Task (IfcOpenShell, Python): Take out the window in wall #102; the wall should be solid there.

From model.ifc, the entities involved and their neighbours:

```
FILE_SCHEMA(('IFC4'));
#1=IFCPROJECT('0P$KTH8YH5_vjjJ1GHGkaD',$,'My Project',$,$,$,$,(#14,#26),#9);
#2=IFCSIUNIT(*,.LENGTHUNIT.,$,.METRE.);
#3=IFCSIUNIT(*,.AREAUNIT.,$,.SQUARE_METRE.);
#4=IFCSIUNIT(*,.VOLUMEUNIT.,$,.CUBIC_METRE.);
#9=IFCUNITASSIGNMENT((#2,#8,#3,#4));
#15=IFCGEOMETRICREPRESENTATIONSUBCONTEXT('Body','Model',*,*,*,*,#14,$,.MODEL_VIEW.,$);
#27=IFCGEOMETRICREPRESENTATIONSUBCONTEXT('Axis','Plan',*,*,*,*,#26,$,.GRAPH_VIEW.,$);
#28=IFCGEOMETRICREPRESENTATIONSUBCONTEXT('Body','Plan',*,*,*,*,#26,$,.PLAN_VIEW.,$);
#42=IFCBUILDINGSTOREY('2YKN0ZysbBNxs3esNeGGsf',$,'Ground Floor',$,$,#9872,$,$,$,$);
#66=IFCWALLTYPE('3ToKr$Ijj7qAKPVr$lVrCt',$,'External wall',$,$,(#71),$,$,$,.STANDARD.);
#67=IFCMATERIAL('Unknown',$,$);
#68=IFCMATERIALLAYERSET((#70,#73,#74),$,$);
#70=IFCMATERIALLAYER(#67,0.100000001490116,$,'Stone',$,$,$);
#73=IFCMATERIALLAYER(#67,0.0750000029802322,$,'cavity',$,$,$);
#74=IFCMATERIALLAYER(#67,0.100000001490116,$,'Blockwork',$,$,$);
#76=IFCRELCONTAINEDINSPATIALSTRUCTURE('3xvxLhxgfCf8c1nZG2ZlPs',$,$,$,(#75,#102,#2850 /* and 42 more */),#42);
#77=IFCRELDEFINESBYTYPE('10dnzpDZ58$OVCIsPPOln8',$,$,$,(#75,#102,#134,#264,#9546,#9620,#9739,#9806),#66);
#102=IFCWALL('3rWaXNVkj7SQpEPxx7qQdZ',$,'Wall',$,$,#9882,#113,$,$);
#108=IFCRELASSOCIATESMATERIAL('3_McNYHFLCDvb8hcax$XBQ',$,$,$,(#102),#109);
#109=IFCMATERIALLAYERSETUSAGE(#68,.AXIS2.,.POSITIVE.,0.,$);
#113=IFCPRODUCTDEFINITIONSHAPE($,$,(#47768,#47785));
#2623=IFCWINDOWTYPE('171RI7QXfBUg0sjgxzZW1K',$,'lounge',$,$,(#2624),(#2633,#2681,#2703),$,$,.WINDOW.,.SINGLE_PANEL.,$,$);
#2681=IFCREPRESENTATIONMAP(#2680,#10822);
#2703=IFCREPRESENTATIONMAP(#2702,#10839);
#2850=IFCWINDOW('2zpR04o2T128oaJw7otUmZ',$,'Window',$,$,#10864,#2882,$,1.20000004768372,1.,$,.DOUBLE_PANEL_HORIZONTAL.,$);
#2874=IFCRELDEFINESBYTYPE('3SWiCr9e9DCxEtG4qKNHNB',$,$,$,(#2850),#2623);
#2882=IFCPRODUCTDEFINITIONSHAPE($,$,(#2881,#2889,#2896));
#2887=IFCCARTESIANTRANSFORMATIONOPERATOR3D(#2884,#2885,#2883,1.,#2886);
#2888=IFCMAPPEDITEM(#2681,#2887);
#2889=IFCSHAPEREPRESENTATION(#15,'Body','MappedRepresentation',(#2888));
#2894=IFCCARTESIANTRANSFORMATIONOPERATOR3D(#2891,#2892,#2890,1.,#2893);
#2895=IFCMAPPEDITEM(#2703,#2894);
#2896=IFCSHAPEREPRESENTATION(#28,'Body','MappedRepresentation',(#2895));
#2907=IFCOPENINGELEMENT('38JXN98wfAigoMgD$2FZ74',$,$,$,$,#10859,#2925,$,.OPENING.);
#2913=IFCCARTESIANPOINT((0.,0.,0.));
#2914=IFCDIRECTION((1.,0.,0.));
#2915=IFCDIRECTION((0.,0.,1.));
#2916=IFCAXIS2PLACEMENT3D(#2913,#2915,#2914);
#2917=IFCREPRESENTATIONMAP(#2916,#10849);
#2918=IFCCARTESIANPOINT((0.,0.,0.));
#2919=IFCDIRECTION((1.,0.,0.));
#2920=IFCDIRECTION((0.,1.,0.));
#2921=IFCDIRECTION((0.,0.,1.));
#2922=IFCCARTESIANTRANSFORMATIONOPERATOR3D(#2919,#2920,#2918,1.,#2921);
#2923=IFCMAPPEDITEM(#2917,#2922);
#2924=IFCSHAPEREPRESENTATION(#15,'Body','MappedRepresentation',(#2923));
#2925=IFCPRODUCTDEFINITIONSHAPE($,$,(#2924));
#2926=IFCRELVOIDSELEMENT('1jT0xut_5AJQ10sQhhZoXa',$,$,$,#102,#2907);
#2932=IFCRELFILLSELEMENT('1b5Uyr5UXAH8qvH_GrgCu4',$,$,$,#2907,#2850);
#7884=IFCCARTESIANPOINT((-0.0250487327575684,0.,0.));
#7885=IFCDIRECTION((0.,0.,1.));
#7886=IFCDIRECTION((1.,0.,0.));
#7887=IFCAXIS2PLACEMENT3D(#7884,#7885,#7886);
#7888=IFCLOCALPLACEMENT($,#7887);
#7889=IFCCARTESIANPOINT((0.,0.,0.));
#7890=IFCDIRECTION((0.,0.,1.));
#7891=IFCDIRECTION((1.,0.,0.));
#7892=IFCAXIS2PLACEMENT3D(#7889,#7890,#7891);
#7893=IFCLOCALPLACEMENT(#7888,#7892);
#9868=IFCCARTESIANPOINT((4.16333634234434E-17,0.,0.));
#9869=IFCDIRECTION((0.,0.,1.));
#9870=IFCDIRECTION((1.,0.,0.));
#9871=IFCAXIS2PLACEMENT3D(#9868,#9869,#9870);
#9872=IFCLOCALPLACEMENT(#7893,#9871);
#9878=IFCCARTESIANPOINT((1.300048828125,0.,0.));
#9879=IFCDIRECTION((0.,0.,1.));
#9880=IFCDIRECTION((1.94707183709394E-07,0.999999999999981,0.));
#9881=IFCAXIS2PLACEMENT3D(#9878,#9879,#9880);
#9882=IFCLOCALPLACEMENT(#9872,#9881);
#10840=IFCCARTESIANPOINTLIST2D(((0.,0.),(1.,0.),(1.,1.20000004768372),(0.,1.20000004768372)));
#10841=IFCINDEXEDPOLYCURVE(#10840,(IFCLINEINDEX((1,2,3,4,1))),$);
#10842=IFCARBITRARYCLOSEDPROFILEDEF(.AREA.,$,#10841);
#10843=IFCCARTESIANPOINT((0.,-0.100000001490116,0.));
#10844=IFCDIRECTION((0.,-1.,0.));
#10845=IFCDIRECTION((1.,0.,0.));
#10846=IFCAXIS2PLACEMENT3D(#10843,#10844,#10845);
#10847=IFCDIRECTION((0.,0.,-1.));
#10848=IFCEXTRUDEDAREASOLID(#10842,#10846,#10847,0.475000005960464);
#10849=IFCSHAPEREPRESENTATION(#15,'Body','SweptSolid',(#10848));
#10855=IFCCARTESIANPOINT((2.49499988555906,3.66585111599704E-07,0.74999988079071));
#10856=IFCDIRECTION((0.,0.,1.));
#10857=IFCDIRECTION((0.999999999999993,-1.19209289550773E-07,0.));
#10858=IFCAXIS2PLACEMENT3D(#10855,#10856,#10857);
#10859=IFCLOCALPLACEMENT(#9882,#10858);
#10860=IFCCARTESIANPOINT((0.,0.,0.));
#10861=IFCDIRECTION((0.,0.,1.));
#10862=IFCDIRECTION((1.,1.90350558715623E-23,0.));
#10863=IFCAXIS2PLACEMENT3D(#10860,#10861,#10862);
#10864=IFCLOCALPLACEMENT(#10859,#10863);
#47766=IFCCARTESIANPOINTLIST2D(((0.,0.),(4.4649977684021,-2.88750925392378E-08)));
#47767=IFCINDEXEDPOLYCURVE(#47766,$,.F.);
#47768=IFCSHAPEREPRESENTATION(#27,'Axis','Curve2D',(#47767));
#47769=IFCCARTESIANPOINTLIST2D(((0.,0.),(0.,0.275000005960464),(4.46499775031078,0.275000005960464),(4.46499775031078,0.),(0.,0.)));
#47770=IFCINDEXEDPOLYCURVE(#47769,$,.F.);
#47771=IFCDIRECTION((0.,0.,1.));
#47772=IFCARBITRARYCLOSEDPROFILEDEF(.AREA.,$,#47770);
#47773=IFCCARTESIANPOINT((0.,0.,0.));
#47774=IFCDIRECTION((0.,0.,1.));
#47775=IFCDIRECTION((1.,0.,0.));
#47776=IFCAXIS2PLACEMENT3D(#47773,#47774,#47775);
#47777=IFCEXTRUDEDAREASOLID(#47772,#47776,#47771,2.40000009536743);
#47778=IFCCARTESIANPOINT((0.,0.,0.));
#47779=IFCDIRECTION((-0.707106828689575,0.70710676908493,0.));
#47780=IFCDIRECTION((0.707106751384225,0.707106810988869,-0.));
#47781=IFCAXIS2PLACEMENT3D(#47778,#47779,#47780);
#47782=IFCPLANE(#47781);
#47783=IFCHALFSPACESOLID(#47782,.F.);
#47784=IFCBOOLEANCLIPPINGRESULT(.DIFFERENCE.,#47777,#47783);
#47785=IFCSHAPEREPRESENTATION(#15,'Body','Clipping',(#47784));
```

```python
import ifcopenshell
import ifcopenshell.api.feature
import ifcopenshell.api.root
import ifcopenshell.geom
import ifcopenshell.util.shape

model = ifcopenshell.open("model.ifc")
settings = ifcopenshell.geom.settings()


def volume(element):
    """Net volume in cubic metres, openings subtracted."""
    shape = ifcopenshell.geom.create_shape(settings, element)
    return ifcopenshell.util.shape.get_volume(shape.geometry)


window = model.by_guid("2zpR04o2T128oaJw7otUmZ")
opening = window.FillsVoids[0].RelatingOpeningElement
wall = opening.VoidsElements[0].RelatingBuildingElement
before = volume(wall)

ifcopenshell.api.root.remove_product(model, product=window)
ifcopenshell.api.feature.remove_feature(model, feature=opening)

after = volume(wall)

print(f"wall volume {before:.3f} -> {after:.3f} m3")

model.write("model-out.ifc")
```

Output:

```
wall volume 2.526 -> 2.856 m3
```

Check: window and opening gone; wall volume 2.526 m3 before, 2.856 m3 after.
